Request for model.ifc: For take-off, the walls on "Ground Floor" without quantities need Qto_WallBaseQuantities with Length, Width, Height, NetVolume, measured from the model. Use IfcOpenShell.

First a look at what the model holds.

```python
import ifcopenshell
import ifcopenshell.util.element
import ifcopenshell.util.unit

model = ifcopenshell.open("model.ifc")
print(model.schema)
for unit_type in ("LENGTHUNIT", "AREAUNIT", "VOLUMEUNIT"):
    print(unit_type, ifcopenshell.util.unit.calculate_unit_scale(model, unit_type))
storey = next(s for s in model.by_type("IfcBuildingStorey") if s.Name == "Ground Floor")
walls = [e for e in ifcopenshell.util.element.get_decomposition(storey) if e.is_a("IfcWall")]
for e in sorted(walls, key=lambda e: e.id()):
    print(e.id(), e.is_a(), e.Name, list(ifcopenshell.util.element.get_psets(e, qtos_only=True)), sep=" | ")
```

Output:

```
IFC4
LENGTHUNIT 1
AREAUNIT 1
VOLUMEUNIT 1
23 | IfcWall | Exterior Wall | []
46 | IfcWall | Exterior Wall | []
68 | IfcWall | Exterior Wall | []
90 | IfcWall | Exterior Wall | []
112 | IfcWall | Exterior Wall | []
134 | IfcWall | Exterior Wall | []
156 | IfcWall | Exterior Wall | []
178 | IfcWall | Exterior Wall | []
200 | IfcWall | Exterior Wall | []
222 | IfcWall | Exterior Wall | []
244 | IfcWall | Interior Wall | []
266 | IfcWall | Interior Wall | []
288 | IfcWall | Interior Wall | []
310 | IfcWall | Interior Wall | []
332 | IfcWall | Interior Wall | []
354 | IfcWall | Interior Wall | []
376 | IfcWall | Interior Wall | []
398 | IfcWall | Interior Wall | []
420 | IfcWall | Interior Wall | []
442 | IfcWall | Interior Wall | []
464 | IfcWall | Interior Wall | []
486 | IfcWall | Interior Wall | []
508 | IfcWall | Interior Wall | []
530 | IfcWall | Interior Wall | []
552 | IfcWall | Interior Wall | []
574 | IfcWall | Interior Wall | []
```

```python
import ifcopenshell
import ifcopenshell.api.pset
import ifcopenshell.geom
import ifcopenshell.util.element
import ifcopenshell.util.shape
import ifcopenshell.util.unit

model = ifcopenshell.open("model.ifc")
unit_scale = ifcopenshell.util.unit.calculate_unit_scale(model)
volume_scale = ifcopenshell.util.unit.calculate_unit_scale(model, "VOLUMEUNIT")
settings = ifcopenshell.geom.settings()

storey = next(s for s in model.by_type("IfcBuildingStorey") if s.Name == "Ground Floor")
walls = [e for e in ifcopenshell.util.element.get_decomposition(storey) if e.is_a("IfcWall")]

for e in sorted(walls, key=lambda e: e.id()):
    if ifcopenshell.util.element.get_psets(e, qtos_only=True, should_inherit=False):
        continue
    # Geometry comes back in metres, in the element's own axes.
    shape = ifcopenshell.geom.create_shape(settings, e)
    values = {
        "Length": ifcopenshell.util.shape.get_x(shape.geometry) / unit_scale,
        "Width": ifcopenshell.util.shape.get_y(shape.geometry) / unit_scale,
        "Height": ifcopenshell.util.shape.get_z(shape.geometry) / unit_scale,
        "NetVolume": ifcopenshell.util.shape.get_volume(shape.geometry) / volume_scale,
    }
    qto = ifcopenshell.api.pset.add_qto(model, product=e, name="Qto_WallBaseQuantities")
    ifcopenshell.api.pset.edit_qto(model, qto=qto, properties=values)
    print(e.id(), {k: round(v, 3) for k, v in values.items()})

model.write("model_edited.ifc")
```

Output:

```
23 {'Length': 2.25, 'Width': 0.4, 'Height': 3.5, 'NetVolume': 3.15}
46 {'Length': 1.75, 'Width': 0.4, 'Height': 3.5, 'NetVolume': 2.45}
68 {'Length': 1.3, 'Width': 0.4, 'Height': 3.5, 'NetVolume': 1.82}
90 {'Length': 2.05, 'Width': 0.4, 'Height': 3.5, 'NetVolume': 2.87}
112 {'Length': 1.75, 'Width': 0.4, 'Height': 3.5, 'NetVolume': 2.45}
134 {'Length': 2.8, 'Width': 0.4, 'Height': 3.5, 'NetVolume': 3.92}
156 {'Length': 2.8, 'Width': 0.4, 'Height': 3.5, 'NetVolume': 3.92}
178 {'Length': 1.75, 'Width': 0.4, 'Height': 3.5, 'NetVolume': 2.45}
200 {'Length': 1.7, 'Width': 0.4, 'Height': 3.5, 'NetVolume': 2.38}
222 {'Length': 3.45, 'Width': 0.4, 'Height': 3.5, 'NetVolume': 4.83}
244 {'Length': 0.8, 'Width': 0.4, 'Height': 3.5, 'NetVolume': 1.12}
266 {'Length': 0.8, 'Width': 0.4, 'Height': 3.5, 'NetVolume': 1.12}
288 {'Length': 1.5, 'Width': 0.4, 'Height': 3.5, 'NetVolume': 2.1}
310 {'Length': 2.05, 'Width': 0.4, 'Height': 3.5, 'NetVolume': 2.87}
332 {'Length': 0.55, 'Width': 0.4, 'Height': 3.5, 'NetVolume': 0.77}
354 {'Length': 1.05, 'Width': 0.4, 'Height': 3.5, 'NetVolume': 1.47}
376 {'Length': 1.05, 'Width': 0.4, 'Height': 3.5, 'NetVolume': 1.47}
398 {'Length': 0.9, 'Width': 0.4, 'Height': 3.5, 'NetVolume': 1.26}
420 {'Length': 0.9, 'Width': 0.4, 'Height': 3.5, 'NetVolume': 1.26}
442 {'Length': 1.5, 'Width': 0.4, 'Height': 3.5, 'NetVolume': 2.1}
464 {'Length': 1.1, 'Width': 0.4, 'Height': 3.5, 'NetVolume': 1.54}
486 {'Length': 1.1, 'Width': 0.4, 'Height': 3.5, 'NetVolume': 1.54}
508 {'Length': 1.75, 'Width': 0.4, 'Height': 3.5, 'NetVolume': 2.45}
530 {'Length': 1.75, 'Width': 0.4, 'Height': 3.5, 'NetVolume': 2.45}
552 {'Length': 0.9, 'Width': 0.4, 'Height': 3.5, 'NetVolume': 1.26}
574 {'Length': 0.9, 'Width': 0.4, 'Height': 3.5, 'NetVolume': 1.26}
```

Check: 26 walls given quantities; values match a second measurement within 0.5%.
